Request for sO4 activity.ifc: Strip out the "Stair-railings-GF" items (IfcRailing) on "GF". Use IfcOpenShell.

First a look at what the model holds.

```python
import ifcopenshell
import ifcopenshell.util.element

model = ifcopenshell.open("sO4 activity.ifc")
print(model.schema)
storey = next(s for s in model.by_type("IfcBuildingStorey") if s.Name == "GF")
railings = [e for e in ifcopenshell.util.element.get_decomposition(storey) if e.is_a("IfcRailing")]
seen = {}
for e in railings:
    element_type = ifcopenshell.util.element.get_type(e)
    name = element_type.Name if element_type not in (None, e) else None
    seen[name] = seen.get(name, 0) + 1
for name, count in sorted(seen.items(), key=str):
    print(count, "x", name)
```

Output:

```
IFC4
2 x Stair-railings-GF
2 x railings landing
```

```python
import ifcopenshell
import ifcopenshell.api.root
import ifcopenshell.util.element

model = ifcopenshell.open("sO4 activity.ifc")

storey = next(s for s in model.by_type("IfcBuildingStorey") if s.Name == "GF")
railings = [e for e in ifcopenshell.util.element.get_decomposition(storey) if e.is_a("IfcRailing")]
targets = [e for e in railings if (t := ifcopenshell.util.element.get_type(e)) not in (None, e) and t.Name == "Stair-railings-GF"]

for e in targets:
    ifcopenshell.api.root.remove_product(model, product=e)
print(len(targets), "removed")

model.write("sO4 activity-out.ifc")
```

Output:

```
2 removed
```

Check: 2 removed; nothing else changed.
